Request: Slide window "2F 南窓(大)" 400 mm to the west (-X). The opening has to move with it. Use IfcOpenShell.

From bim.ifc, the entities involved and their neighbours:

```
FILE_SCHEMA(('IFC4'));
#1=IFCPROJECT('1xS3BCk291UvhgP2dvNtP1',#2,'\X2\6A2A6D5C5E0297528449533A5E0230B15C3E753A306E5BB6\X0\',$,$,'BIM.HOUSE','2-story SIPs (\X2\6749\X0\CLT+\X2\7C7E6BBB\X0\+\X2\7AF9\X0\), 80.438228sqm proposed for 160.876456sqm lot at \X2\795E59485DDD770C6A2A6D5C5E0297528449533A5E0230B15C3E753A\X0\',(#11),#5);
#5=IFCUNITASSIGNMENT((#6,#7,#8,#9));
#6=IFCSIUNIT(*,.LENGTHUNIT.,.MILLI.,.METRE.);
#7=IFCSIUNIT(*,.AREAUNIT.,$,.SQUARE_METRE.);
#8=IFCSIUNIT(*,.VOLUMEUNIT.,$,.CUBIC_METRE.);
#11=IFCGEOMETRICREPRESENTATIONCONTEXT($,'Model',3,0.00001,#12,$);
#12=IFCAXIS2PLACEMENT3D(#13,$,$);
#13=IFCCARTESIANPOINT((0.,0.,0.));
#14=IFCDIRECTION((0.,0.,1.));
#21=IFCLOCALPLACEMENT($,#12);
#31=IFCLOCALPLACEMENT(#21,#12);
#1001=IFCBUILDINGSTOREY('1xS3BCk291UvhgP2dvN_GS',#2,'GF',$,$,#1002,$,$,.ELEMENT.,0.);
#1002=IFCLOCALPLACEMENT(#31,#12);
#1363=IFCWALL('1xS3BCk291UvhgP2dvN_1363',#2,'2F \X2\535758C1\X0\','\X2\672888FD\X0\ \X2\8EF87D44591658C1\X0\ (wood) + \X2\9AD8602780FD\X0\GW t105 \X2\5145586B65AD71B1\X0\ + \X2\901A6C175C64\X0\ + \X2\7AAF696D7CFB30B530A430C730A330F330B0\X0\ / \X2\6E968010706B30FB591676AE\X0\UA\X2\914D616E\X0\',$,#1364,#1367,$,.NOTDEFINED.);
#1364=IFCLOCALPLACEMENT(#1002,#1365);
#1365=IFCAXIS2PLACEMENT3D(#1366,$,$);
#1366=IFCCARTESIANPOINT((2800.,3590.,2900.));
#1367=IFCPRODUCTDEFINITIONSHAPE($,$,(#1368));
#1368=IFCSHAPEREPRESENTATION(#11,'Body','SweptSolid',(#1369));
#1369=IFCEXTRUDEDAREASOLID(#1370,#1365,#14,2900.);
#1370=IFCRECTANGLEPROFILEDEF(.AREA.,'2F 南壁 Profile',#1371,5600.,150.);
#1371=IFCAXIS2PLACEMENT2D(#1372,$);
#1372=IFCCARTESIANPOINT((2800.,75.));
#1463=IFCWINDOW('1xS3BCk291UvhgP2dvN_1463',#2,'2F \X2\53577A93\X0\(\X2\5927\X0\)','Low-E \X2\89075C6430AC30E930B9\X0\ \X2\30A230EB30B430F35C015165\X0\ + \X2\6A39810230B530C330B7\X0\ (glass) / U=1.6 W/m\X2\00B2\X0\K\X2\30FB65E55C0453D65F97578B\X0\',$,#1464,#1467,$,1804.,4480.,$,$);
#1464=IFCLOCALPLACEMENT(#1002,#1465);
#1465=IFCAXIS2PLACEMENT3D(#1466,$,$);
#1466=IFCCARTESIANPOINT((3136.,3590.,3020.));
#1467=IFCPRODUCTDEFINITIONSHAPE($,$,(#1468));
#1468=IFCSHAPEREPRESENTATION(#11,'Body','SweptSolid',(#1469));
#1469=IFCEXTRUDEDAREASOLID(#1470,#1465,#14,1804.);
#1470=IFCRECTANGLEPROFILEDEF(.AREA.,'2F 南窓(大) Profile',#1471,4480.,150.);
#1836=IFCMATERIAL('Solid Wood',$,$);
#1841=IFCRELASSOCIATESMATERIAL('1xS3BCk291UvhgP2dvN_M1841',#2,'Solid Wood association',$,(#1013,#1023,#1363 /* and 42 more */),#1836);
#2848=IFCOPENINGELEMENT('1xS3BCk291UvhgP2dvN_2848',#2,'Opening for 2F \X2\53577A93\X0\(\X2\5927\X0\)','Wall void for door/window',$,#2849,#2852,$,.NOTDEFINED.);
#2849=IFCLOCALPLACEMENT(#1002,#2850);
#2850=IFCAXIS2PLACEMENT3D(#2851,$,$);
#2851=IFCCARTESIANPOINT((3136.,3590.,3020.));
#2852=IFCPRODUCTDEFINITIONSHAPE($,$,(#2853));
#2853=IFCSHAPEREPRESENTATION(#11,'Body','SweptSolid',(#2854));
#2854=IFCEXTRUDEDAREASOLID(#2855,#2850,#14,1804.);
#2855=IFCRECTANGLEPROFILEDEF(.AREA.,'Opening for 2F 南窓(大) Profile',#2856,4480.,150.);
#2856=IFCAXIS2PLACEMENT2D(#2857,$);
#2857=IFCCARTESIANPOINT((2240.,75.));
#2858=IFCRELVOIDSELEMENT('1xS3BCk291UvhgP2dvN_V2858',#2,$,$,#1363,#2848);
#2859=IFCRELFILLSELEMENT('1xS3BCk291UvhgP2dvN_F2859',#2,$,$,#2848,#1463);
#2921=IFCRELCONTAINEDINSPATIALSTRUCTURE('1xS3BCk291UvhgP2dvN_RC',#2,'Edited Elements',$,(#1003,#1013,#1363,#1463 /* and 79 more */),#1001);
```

```python
import ifcopenshell
import ifcopenshell.api.geometry
import ifcopenshell.util.placement
import ifcopenshell.util.unit

model = ifcopenshell.open("bim.ifc")
unit_scale = ifcopenshell.util.unit.calculate_unit_scale(model)

window = model.by_guid("1xS3BCk291UvhgP2dvN_1463")
opening = window.FillsVoids[0].RelatingOpeningElement
wall = opening.VoidsElements[0].RelatingBuildingElement

wall_matrix = ifcopenshell.util.placement.get_local_placement(wall.ObjectPlacement)
shift = wall_matrix[:3, 0] * -0.4 / unit_scale
before = ifcopenshell.util.placement.get_local_placement(window.ObjectPlacement)[:3, 3].copy()

# The window is not placed relative to its opening, so move both.
for product in (opening, window):
    matrix = ifcopenshell.util.placement.get_local_placement(product.ObjectPlacement)
    matrix[:3, 3] += shift
    ifcopenshell.api.geometry.edit_object_placement(model, product=product, matrix=matrix, is_si=False)

after = ifcopenshell.util.placement.get_local_placement(window.ObjectPlacement)[:3, 3]
print("window moved by", (after - before).round(3) + 0.0)

model.write("bim_rev.ifc")
```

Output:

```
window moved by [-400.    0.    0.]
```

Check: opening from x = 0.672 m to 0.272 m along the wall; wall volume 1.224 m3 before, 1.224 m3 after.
